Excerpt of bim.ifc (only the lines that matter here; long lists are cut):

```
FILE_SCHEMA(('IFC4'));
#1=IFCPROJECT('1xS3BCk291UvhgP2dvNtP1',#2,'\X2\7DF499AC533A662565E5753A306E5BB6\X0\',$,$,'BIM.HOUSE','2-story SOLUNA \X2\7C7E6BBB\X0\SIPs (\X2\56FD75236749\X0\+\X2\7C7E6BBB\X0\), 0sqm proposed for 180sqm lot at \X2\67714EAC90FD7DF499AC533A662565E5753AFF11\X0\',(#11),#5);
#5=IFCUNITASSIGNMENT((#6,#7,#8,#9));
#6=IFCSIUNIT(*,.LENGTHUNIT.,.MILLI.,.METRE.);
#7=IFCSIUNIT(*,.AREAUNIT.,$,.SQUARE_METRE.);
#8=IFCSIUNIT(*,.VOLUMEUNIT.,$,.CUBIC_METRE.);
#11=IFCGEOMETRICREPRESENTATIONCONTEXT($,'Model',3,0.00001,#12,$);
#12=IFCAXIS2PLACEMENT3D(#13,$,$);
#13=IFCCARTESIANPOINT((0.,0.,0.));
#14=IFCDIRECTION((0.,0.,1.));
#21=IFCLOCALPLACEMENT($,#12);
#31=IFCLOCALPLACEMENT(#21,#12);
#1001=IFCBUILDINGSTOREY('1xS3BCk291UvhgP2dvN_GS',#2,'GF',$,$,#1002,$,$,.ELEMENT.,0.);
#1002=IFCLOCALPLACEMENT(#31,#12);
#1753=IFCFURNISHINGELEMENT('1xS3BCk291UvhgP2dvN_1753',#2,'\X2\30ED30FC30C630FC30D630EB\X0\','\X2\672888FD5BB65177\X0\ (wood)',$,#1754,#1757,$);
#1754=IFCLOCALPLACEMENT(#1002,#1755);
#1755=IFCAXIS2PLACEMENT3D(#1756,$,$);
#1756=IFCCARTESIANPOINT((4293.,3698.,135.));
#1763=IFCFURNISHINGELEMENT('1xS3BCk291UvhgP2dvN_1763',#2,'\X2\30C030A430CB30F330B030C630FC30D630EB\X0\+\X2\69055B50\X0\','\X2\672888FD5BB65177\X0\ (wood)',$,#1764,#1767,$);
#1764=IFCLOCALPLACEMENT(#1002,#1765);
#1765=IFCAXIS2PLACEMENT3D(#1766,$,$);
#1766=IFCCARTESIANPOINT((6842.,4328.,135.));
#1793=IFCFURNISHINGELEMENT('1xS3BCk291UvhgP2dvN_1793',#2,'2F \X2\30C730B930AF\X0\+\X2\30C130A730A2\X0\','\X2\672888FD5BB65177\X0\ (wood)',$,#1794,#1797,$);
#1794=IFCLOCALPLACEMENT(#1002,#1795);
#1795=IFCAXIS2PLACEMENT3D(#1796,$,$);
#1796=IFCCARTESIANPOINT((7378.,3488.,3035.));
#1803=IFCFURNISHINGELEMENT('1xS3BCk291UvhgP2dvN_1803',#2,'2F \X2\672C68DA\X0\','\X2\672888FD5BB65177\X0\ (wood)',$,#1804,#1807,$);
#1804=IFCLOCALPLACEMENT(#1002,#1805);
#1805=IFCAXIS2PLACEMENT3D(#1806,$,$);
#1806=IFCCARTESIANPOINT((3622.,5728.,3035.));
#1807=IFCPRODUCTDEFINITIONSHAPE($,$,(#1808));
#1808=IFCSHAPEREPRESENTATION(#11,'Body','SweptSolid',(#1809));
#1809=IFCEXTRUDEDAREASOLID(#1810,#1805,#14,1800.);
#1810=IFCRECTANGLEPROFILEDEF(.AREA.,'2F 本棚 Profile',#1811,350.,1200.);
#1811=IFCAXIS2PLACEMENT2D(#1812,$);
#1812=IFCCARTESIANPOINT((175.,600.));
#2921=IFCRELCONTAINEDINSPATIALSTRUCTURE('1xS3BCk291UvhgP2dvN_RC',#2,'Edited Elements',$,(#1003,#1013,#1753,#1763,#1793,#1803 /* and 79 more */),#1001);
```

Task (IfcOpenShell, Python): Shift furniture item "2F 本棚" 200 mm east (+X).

```python
import ifcopenshell
import ifcopenshell.api.geometry
import ifcopenshell.util.placement

model = ifcopenshell.open("bim.ifc")

item = model.by_guid("1xS3BCk291UvhgP2dvN_1803")
matrix = ifcopenshell.util.placement.get_local_placement(item.ObjectPlacement)
matrix[0, 3] += 200.0
ifcopenshell.api.geometry.edit_object_placement(model, product=item, matrix=matrix, is_si=False)

print(ifcopenshell.util.placement.get_local_placement(item.ObjectPlacement).round(3) + 0.0)

model.write("bim_edited.ifc")
```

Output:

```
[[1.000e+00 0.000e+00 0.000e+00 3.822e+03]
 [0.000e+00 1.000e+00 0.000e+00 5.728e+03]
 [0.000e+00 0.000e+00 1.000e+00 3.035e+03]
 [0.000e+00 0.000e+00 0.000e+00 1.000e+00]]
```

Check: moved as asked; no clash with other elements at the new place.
